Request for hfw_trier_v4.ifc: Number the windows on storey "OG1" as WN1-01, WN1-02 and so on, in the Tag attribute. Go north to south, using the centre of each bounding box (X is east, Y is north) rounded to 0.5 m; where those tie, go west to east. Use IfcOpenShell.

First a look at what the model holds.

```python
import ifcopenshell
import ifcopenshell.util.element
import ifcopenshell.util.placement

model = ifcopenshell.open("hfw_trier_v4.ifc")
print(model.schema)
storey = next(s for s in model.by_type("IfcBuildingStorey") if s.Name == "OG1")
windows = [e for e in ifcopenshell.util.element.get_decomposition(storey) if e.is_a("IfcWindow")]
for e in sorted(windows, key=lambda e: e.id()):
    origin = ifcopenshell.util.placement.get_local_placement(e.ObjectPlacement)[:3, 3]
    print(e.id(), e.Tag, e.Name, origin.round(2) + 0.0, sep=" | ")
```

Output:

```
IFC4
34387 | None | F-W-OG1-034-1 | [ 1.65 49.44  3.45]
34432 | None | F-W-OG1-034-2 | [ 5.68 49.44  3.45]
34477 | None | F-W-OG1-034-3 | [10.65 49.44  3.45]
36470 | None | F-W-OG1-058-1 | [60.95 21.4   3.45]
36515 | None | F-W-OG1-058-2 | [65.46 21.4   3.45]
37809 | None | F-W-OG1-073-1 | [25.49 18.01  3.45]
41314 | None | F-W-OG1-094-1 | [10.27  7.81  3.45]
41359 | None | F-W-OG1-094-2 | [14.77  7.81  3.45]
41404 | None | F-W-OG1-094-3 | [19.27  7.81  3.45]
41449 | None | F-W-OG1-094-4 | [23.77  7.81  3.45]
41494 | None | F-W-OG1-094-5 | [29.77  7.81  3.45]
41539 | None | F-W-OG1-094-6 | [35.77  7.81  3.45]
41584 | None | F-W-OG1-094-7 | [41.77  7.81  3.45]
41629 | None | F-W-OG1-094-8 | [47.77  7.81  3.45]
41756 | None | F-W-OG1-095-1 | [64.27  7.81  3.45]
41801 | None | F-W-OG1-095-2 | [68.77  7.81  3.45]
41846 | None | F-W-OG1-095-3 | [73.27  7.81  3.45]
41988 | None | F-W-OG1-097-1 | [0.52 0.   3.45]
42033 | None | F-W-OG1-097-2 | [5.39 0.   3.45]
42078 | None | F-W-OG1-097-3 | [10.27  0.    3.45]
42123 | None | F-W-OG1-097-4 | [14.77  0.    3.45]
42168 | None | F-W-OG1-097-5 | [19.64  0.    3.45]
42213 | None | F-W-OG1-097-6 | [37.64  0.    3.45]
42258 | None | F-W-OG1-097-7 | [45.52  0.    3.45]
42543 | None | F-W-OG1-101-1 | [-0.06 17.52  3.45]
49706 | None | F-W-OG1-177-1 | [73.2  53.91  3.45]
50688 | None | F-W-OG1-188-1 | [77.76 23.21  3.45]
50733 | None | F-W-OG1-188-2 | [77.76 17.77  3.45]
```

```python
import ifcopenshell
import ifcopenshell.geom
import ifcopenshell.util.element
import ifcopenshell.util.shape

model = ifcopenshell.open("hfw_trier_v4.ifc")
settings = ifcopenshell.geom.settings()
settings.set("use-world-coords", True)


def centre(element):
    shape = ifcopenshell.geom.create_shape(settings, element)
    return ifcopenshell.util.shape.get_bbox_centroid(shape.geometry)


storey = next(s for s in model.by_type("IfcBuildingStorey") if s.Name == "OG1")
windows = [e for e in ifcopenshell.util.element.get_decomposition(storey) if e.is_a("IfcWindow")]

# Insertion points can sit at a corner or the storey origin, so sort by the geometry (in metres).
centres = {e: centre(e) for e in windows}
windows.sort(key=lambda e: (-round(centres[e][1] / 0.5), centres[e][0]))

for i, e in enumerate(windows, start=1):
    number = f"WN1-{i:02d}"
    e.Tag = number
    print(e.id(), number)

model.write("hfw_trier_v4_edited.ifc")
```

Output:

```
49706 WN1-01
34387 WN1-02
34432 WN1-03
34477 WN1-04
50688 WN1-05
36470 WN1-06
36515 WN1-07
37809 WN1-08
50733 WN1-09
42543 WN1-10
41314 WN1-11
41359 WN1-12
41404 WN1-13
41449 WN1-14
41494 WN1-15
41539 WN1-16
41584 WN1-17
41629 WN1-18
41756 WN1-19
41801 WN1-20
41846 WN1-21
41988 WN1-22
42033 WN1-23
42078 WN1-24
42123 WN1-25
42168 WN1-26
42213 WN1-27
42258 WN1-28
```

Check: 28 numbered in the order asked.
